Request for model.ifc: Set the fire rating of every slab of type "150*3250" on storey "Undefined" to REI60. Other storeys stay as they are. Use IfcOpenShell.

First a look at what the model holds.

```python
import ifcopenshell
import ifcopenshell.util.element

model = ifcopenshell.open("model.ifc")
print(model.schema)
storey = next(s for s in model.by_type("IfcBuildingStorey") if s.Name == "Undefined")
slabs = [e for e in ifcopenshell.util.element.get_decomposition(storey) if e.is_a("IfcSlab")]
seen = {}
for e in slabs:
    element_type = ifcopenshell.util.element.get_type(e)
    key = (element_type.Name if element_type != e and element_type else None, ifcopenshell.util.element.get_pset(e, "Pset_SlabCommon", "FireRating"))
    seen[key] = seen.get(key, 0) + 1
for (name, value), count in sorted(seen.items(), key=str):
    print(count, "x", name, "|", value)
```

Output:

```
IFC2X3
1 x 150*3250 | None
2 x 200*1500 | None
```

```python
import ifcopenshell
import ifcopenshell.api.pset
import ifcopenshell.util.element

model = ifcopenshell.open("model.ifc")

storey = next(s for s in model.by_type("IfcBuildingStorey") if s.Name == "Undefined")
slabs = [e for e in ifcopenshell.util.element.get_decomposition(storey) if e.is_a("IfcSlab")]

count = 0
for e in slabs:
    element_type = ifcopenshell.util.element.get_type(e)
    if element_type in (None, e) or element_type.Name != "150*3250":
        continue
    # add_pset returns the element's existing set when there is one.
    pset = ifcopenshell.api.pset.add_pset(model, product=e, name="Pset_SlabCommon")
    ifcopenshell.api.pset.edit_pset(model, pset=pset, properties={"FireRating": "REI60"})
    count += 1

print(count, "slabs updated")

model.write("model_rev.ifc")
```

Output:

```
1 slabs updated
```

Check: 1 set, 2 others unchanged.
